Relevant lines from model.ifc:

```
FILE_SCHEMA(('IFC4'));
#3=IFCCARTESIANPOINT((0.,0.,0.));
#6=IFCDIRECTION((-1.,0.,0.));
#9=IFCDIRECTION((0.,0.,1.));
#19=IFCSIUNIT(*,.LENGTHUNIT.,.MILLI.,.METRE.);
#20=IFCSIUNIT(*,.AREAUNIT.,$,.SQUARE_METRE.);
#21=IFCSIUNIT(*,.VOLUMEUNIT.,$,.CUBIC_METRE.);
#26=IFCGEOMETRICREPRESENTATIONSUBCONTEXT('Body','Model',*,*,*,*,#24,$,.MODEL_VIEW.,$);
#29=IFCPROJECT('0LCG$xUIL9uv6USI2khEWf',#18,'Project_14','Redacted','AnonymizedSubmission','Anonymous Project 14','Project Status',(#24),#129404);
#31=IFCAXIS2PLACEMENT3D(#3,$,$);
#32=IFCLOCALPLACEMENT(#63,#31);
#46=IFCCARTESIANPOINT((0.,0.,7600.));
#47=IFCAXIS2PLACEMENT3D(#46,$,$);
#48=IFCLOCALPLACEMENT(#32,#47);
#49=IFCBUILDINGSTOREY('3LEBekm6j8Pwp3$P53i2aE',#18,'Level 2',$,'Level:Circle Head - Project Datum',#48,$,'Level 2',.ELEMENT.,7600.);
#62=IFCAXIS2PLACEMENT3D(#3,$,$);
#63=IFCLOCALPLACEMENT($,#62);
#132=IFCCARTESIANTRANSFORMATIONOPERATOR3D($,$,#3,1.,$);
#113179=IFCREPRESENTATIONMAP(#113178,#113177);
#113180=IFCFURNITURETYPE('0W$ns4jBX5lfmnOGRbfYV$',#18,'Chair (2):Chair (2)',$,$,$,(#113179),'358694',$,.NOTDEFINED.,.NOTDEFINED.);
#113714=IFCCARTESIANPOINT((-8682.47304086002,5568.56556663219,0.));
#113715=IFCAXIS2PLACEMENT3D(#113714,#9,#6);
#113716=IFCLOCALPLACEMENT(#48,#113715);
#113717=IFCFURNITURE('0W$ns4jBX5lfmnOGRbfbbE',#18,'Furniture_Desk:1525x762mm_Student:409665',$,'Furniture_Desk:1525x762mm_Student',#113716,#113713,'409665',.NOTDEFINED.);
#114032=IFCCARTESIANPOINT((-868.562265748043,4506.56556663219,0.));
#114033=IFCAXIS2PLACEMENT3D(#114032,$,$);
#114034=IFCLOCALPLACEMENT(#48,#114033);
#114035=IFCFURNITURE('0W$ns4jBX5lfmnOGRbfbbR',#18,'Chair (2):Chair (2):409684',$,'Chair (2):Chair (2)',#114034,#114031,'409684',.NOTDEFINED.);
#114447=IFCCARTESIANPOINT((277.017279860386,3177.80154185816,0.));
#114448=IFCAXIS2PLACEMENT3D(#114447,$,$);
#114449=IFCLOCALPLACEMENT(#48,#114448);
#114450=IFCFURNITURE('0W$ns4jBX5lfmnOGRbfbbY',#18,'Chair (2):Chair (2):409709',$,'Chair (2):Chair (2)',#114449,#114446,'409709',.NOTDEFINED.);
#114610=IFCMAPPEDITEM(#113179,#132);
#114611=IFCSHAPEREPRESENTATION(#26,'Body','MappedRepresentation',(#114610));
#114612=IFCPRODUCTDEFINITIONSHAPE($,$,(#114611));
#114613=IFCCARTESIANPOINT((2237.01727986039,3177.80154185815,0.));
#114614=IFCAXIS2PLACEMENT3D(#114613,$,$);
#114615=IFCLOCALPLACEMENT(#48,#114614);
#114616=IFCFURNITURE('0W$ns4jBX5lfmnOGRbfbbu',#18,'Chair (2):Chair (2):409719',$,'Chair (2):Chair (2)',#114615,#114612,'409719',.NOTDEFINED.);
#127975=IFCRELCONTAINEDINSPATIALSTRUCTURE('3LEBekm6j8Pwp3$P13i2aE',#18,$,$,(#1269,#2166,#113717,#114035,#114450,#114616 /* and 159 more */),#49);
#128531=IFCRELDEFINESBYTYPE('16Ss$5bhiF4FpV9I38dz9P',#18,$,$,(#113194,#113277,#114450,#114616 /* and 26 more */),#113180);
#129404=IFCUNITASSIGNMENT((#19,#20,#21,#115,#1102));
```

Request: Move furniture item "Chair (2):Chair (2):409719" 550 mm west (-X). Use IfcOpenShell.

```python
import ifcopenshell
import ifcopenshell.api.geometry
import ifcopenshell.util.placement

model = ifcopenshell.open("model.ifc")

item = model.by_guid("0W$ns4jBX5lfmnOGRbfbbu")
matrix = ifcopenshell.util.placement.get_local_placement(item.ObjectPlacement)
matrix[0, 3] -= 550.0
ifcopenshell.api.geometry.edit_object_placement(model, product=item, matrix=matrix, is_si=False)

print(ifcopenshell.util.placement.get_local_placement(item.ObjectPlacement).round(3) + 0.0)

model.write("model_updated.ifc")
```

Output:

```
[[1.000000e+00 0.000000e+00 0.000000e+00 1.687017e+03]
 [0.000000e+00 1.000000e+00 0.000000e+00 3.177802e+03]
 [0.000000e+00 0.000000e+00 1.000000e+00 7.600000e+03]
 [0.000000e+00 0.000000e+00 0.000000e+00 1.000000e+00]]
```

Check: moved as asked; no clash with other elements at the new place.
